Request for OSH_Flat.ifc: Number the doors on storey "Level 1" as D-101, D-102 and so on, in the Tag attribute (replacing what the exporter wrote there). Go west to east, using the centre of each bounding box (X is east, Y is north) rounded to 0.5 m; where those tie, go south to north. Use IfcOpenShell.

First a look at what the model holds.

```python
import ifcopenshell
import ifcopenshell.util.element
import ifcopenshell.util.placement

model = ifcopenshell.open("OSH_Flat.ifc")
print(model.schema)
storey = next(s for s in model.by_type("IfcBuildingStorey") if s.Name == "Level 1")
doors = [e for e in ifcopenshell.util.element.get_decomposition(storey) if e.is_a("IfcDoor")]
for e in sorted(doors, key=lambda e: e.id()):
    origin = ifcopenshell.util.placement.get_local_placement(e.ObjectPlacement)[:3, 3]
    print(e.id(), e.Tag, e.Name, origin.round(2) + 0.0, sep=" | ")
```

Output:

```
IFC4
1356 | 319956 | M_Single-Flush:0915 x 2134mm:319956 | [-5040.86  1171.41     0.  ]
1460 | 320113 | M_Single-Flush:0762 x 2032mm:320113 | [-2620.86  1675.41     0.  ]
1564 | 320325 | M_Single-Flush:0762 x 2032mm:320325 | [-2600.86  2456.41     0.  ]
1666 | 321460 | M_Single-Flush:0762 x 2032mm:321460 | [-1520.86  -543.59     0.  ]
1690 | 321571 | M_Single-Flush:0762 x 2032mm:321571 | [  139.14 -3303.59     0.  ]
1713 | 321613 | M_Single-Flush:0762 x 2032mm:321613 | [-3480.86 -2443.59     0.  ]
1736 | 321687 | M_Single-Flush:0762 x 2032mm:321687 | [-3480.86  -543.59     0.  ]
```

```python
import ifcopenshell
import ifcopenshell.geom
import ifcopenshell.util.element
import ifcopenshell.util.shape

model = ifcopenshell.open("OSH_Flat.ifc")
settings = ifcopenshell.geom.settings()
settings.set("use-world-coords", True)


def centre(element):
    shape = ifcopenshell.geom.create_shape(settings, element)
    return ifcopenshell.util.shape.get_bbox_centroid(shape.geometry)


storey = next(s for s in model.by_type("IfcBuildingStorey") if s.Name == "Level 1")
doors = [e for e in ifcopenshell.util.element.get_decomposition(storey) if e.is_a("IfcDoor")]

# Insertion points can sit at a corner or the storey origin, so sort by the geometry (in metres).
centres = {e: centre(e) for e in doors}
doors.sort(key=lambda e: (round(centres[e][0] / 0.5), centres[e][1]))

for i, e in enumerate(doors, start=1):
    number = f"D-1{i:02d}"
    e.Tag = number
    print(e.id(), number)

model.write("OSH_Flat_rev.ifc")
```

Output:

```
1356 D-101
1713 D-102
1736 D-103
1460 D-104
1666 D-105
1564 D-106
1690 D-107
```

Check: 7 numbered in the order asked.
